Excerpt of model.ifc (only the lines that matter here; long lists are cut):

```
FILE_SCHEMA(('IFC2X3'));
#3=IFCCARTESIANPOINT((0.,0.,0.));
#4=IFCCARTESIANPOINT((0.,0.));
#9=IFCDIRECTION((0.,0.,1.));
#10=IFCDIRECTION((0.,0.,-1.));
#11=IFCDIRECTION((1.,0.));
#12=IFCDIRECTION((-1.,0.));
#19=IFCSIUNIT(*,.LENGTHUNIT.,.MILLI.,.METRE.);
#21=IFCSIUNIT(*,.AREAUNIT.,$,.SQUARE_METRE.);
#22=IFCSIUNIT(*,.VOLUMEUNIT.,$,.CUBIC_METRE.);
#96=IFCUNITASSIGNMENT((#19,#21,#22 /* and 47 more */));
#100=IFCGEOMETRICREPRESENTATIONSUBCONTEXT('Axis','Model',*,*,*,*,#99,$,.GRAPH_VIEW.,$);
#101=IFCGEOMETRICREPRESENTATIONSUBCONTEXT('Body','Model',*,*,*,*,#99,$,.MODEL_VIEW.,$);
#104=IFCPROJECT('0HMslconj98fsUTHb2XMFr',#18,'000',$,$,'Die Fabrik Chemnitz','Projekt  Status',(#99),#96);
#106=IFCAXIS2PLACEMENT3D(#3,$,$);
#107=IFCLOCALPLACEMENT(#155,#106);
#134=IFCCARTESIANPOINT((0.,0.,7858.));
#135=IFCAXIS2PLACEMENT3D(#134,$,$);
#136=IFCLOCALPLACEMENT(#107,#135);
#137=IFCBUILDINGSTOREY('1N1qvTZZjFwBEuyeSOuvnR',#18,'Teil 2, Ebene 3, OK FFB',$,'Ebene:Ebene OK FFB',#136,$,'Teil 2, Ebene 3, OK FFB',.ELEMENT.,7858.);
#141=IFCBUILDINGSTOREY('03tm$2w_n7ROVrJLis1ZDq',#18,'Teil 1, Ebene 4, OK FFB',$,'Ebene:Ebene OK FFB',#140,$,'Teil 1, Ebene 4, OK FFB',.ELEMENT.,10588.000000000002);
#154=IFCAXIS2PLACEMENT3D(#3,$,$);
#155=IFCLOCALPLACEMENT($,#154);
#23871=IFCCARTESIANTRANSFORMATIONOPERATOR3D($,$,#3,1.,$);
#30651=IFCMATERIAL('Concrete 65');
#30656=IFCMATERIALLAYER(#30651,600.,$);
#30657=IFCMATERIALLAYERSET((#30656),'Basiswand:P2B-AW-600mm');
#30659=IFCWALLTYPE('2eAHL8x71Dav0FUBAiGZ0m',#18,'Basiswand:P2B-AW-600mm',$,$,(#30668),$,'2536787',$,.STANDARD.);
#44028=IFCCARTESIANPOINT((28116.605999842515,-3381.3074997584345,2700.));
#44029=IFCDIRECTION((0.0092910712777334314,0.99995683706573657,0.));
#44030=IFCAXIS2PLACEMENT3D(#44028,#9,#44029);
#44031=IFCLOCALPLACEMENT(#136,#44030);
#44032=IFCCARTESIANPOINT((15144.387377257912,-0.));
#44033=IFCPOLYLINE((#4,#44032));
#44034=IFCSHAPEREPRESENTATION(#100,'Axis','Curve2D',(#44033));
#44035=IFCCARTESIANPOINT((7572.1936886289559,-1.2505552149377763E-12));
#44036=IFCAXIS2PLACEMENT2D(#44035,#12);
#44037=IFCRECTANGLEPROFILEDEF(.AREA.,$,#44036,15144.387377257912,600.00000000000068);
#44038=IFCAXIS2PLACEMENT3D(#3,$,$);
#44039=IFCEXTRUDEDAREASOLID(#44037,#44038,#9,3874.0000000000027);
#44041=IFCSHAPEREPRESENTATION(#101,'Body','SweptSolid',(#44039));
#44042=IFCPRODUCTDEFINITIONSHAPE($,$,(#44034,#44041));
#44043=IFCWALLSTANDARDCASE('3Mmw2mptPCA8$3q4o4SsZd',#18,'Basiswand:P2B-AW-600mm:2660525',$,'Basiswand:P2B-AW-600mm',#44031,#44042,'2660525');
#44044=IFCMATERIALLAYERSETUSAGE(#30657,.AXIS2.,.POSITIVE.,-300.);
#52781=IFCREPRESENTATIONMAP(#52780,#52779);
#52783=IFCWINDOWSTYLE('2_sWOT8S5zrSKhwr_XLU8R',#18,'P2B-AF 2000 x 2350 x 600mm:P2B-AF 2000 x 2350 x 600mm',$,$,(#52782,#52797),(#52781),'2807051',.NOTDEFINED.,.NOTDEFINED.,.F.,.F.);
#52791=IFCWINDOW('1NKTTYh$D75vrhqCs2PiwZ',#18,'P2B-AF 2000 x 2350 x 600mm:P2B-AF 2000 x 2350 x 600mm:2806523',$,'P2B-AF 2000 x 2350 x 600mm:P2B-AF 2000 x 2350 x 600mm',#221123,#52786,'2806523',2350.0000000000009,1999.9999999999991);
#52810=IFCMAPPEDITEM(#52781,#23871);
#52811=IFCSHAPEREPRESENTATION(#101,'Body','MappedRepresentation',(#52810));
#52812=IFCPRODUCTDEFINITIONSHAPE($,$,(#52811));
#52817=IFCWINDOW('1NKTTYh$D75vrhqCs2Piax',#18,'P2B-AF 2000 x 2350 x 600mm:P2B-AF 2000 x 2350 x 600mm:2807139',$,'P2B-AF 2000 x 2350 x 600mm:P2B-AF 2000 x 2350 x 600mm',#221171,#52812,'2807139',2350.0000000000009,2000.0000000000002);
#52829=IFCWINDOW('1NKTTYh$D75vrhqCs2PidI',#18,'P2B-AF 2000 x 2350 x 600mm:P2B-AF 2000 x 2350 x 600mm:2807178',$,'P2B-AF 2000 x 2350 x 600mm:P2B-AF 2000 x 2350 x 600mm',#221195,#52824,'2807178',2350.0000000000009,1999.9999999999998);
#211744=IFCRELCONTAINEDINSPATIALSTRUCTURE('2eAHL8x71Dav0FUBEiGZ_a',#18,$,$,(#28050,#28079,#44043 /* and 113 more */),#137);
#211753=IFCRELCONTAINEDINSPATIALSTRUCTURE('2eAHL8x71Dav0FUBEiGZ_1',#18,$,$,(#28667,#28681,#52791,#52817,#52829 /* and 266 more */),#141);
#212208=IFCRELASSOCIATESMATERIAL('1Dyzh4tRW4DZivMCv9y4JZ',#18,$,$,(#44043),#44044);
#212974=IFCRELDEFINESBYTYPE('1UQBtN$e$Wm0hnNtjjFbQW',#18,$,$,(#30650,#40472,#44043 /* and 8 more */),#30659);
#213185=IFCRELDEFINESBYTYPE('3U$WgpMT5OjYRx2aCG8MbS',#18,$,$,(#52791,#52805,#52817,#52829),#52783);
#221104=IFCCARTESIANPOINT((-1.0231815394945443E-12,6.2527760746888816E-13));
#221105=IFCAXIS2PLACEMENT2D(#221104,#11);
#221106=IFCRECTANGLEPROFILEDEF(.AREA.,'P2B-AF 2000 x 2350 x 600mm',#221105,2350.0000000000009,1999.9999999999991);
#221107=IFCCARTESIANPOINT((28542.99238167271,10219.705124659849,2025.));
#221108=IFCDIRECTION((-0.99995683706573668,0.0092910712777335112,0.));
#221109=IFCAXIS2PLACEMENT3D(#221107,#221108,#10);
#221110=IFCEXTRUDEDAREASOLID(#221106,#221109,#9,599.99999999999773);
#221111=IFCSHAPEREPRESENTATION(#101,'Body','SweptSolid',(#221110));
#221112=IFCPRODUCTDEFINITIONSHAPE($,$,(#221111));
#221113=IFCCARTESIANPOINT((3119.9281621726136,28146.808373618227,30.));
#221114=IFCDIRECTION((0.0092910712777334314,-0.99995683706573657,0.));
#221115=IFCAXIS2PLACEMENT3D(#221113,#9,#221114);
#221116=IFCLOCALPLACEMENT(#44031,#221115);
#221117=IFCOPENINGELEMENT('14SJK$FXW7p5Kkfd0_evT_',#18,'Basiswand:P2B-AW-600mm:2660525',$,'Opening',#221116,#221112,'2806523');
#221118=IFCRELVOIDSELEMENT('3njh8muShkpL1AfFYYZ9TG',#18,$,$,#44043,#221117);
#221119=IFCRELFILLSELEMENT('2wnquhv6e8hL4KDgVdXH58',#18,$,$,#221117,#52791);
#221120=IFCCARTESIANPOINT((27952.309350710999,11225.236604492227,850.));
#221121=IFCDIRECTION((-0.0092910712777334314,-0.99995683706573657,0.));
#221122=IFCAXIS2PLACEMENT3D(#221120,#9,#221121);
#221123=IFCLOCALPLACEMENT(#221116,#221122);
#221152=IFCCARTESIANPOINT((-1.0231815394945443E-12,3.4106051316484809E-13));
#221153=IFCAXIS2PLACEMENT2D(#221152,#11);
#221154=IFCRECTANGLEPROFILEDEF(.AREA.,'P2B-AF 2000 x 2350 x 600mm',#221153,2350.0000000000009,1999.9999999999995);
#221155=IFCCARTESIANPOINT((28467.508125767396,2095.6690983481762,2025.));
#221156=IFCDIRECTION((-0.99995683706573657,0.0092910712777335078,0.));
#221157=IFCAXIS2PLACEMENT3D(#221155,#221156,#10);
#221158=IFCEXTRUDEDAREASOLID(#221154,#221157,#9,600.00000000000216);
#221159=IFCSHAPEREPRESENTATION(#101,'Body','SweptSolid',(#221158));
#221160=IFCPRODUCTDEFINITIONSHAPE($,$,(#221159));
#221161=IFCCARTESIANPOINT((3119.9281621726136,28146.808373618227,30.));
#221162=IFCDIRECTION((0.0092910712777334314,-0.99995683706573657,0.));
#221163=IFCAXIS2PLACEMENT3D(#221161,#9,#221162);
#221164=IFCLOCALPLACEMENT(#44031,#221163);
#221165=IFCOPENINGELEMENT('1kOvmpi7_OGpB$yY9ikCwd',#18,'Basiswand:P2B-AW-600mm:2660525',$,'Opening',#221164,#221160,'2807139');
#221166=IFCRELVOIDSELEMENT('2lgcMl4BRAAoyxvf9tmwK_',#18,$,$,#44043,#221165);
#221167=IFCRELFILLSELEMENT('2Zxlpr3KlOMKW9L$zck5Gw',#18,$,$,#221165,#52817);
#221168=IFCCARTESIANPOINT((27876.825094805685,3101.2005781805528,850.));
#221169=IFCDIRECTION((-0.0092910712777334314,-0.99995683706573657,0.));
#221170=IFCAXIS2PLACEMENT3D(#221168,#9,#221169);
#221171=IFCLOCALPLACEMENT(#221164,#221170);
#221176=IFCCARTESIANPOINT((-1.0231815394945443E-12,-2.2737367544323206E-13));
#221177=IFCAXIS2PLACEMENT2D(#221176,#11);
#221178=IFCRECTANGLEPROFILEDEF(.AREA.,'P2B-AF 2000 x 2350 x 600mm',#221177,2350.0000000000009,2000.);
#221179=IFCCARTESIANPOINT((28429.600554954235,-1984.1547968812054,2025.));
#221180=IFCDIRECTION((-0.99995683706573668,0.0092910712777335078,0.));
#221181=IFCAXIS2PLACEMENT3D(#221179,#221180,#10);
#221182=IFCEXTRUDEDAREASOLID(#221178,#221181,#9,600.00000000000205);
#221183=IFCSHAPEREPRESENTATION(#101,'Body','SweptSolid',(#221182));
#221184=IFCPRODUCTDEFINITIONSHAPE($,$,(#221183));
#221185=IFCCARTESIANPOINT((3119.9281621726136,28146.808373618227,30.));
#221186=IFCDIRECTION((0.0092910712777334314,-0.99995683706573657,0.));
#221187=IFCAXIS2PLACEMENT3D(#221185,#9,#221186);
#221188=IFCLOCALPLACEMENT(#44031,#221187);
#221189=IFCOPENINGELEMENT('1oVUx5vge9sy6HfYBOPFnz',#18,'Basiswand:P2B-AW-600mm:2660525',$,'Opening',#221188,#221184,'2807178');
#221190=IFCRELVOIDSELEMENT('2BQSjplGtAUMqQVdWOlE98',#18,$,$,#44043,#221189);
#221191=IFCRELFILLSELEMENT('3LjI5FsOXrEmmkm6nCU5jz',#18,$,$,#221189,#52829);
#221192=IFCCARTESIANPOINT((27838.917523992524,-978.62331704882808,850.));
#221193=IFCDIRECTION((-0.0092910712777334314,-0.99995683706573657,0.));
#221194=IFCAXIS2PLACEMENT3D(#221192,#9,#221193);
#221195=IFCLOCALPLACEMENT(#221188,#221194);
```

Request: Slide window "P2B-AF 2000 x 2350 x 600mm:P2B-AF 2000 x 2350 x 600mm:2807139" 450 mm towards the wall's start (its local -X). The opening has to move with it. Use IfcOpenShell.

```python
import ifcopenshell
import ifcopenshell.api.geometry
import ifcopenshell.util.placement
import ifcopenshell.util.unit

model = ifcopenshell.open("model.ifc")
unit_scale = ifcopenshell.util.unit.calculate_unit_scale(model)

window = model.by_guid("1NKTTYh$D75vrhqCs2Piax")
opening = window.FillsVoids[0].RelatingOpeningElement
wall = opening.VoidsElements[0].RelatingBuildingElement

wall_matrix = ifcopenshell.util.placement.get_local_placement(wall.ObjectPlacement)
shift = wall_matrix[:3, 0] * -0.45 / unit_scale
before = ifcopenshell.util.placement.get_local_placement(window.ObjectPlacement)[:3, 3].copy()

# The window is placed relative to its opening, so it follows when the opening moves.
matrix = ifcopenshell.util.placement.get_local_placement(opening.ObjectPlacement)
matrix[:3, 3] += shift
ifcopenshell.api.geometry.edit_object_placement(
    model, product=opening, matrix=matrix, is_si=False, should_transform_children=True
)

after = ifcopenshell.util.placement.get_local_placement(window.ObjectPlacement)[:3, 3]
print("window moved by", (after - before).round(3) + 0.0)

model.write("model_updated.ifc")
```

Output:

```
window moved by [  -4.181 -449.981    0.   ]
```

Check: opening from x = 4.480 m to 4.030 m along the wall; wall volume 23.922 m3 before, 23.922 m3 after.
